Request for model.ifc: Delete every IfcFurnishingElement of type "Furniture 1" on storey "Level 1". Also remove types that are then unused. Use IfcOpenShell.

First a look at what the model holds.

```python
import ifcopenshell
import ifcopenshell.util.element

model = ifcopenshell.open("model.ifc")
print(model.schema)
storey = next(s for s in model.by_type("IfcBuildingStorey") if s.Name == "Level 1")
furniture = [e for e in ifcopenshell.util.element.get_decomposition(storey) if e.is_a("IfcFurnishingElement")]
seen = {}
for e in furniture:
    element_type = ifcopenshell.util.element.get_type(e)
    name = element_type.Name if element_type not in (None, e) else None
    seen[name] = seen.get(name, 0) + 1
for name, count in sorted(seen.items(), key=str):
    print(count, "x", name)
```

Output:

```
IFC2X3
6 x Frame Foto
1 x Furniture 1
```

```python
import ifcopenshell
import ifcopenshell.api.root
import ifcopenshell.util.element

model = ifcopenshell.open("model.ifc")

storey = next(s for s in model.by_type("IfcBuildingStorey") if s.Name == "Level 1")
furniture = [e for e in ifcopenshell.util.element.get_decomposition(storey) if e.is_a("IfcFurnishingElement")]
targets = [e for e in furniture if (t := ifcopenshell.util.element.get_type(e)) not in (None, e) and t.Name == "Furniture 1"]
types = {ifcopenshell.util.element.get_type(e) for e in targets} - {None, *targets}

for e in targets:
    ifcopenshell.api.root.remove_product(model, product=e)
print(len(targets), "removed")

unused = [t for t in types if not ifcopenshell.util.element.get_types(t)]
for t in unused:
    ifcopenshell.api.root.remove_product(model, product=t)
print(len(unused), "unused types removed")

model.write("model_edited.ifc")
```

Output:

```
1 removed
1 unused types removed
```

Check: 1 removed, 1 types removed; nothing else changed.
